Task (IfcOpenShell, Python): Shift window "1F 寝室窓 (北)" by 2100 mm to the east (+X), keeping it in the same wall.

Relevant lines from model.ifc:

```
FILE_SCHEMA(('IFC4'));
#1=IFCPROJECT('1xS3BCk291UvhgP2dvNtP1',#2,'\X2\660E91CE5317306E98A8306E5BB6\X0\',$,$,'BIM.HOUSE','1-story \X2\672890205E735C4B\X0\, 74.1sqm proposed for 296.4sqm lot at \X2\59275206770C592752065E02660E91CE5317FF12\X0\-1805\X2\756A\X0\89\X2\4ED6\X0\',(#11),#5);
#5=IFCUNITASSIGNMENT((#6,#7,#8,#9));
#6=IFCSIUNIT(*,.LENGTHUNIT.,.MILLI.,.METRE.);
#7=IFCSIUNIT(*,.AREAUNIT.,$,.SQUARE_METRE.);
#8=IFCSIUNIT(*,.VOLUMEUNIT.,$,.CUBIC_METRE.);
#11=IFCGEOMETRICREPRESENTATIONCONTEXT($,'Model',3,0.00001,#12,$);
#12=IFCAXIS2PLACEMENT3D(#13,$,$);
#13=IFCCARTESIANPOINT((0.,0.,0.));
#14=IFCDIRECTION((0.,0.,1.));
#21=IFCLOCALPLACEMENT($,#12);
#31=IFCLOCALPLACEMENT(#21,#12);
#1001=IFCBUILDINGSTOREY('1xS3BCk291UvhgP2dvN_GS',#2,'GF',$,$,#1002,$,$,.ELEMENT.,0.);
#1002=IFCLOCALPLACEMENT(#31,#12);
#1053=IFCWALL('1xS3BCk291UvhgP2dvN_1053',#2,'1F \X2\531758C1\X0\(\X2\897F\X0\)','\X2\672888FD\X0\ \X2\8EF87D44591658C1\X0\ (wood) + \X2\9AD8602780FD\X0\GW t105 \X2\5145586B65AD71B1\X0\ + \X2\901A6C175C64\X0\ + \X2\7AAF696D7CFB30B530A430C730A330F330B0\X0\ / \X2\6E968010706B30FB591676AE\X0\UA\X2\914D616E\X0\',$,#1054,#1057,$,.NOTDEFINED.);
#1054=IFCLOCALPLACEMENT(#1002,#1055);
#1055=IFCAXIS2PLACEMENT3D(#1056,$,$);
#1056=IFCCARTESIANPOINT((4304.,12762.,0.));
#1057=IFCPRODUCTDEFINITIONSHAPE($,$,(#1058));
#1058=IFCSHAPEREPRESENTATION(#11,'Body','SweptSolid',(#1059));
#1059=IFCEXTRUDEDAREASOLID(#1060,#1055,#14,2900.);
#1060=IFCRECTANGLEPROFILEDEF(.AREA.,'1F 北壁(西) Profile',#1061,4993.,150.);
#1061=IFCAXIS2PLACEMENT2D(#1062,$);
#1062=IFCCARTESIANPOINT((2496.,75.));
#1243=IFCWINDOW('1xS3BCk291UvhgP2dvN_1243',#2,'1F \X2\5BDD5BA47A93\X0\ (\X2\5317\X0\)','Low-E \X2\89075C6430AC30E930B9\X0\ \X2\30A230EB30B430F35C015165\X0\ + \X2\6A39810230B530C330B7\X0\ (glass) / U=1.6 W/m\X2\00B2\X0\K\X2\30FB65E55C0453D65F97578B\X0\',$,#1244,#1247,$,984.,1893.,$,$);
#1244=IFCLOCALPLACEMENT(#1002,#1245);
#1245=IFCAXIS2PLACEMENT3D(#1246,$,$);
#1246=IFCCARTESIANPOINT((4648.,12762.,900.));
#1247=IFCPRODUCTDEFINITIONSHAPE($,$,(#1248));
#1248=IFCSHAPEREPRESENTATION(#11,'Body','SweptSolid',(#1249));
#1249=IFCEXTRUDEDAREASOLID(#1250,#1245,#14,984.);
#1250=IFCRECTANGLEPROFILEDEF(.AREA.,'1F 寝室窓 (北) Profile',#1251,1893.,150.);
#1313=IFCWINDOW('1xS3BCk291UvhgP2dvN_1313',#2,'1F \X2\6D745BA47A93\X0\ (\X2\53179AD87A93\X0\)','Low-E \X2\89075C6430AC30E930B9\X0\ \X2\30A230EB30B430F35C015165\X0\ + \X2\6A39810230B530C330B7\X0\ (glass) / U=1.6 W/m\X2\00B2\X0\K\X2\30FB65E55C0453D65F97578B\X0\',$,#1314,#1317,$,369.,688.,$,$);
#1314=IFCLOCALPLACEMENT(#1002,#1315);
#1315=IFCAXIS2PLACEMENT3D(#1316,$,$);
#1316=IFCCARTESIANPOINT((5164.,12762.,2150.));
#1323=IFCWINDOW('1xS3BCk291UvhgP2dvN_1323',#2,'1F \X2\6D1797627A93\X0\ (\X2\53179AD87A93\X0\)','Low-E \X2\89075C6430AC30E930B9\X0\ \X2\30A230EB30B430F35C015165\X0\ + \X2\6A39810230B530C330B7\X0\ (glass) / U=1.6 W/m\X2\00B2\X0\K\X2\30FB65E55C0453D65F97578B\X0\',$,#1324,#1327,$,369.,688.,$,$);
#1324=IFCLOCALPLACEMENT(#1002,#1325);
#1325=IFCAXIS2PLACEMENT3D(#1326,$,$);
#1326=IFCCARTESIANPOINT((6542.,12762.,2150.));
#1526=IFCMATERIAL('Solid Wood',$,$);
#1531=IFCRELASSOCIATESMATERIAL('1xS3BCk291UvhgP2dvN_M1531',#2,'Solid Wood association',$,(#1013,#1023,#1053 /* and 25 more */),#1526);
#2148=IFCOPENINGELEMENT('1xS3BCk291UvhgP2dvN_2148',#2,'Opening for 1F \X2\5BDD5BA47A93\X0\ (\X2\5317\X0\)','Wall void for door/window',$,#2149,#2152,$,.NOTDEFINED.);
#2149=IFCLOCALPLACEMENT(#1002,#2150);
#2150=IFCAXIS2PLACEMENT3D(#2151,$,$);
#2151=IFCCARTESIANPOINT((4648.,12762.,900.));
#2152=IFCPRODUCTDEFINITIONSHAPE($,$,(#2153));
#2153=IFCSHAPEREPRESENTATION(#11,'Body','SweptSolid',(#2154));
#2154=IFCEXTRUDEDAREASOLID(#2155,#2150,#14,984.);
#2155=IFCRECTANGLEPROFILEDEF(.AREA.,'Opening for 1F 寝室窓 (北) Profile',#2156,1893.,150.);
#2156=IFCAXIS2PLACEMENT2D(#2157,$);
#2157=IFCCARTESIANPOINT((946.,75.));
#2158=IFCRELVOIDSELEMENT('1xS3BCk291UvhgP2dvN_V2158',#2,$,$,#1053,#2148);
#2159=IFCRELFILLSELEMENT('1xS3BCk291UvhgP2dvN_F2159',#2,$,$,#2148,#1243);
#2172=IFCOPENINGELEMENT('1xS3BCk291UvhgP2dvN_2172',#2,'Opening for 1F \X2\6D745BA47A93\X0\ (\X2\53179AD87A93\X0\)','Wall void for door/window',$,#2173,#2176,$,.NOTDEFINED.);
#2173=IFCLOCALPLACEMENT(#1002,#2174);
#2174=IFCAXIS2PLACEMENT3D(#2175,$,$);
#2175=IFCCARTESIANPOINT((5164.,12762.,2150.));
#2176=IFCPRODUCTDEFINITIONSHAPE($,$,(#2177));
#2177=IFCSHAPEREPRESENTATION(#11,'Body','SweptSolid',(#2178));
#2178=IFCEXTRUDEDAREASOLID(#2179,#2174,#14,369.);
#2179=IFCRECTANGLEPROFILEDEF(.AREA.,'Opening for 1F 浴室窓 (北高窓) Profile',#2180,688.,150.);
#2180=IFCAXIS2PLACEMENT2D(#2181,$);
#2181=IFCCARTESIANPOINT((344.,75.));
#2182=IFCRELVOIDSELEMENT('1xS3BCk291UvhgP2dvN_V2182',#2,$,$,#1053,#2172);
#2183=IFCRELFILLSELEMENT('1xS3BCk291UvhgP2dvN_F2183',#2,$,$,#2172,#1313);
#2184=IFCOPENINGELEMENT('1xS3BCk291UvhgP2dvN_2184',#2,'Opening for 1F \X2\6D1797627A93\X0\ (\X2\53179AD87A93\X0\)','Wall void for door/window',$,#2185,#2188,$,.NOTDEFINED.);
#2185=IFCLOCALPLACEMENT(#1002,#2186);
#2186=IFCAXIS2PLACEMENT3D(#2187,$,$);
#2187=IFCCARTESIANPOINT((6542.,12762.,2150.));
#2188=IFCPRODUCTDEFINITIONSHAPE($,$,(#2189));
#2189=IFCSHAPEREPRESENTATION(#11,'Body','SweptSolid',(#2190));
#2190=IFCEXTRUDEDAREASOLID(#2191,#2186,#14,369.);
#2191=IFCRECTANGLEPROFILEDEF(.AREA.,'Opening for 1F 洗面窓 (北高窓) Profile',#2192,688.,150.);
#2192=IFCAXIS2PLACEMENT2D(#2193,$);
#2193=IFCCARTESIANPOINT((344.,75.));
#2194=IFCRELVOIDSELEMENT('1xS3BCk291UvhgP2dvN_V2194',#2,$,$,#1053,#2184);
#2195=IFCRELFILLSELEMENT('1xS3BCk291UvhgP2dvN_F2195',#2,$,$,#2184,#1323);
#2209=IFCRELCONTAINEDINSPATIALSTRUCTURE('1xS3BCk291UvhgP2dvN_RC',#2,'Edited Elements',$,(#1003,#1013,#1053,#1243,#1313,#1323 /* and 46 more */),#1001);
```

```python
import ifcopenshell
import ifcopenshell.api.geometry
import ifcopenshell.util.placement
import ifcopenshell.util.unit

model = ifcopenshell.open("model.ifc")
unit_scale = ifcopenshell.util.unit.calculate_unit_scale(model)

window = model.by_id(1243)
opening = window.FillsVoids[0].RelatingOpeningElement
wall = opening.VoidsElements[0].RelatingBuildingElement

wall_matrix = ifcopenshell.util.placement.get_local_placement(wall.ObjectPlacement)
shift = wall_matrix[:3, 0] * 2.1 / unit_scale
before = ifcopenshell.util.placement.get_local_placement(window.ObjectPlacement)[:3, 3].copy()

# The window is not placed relative to its opening, so move both.
for product in (opening, window):
    matrix = ifcopenshell.util.placement.get_local_placement(product.ObjectPlacement)
    matrix[:3, 3] += shift
    ifcopenshell.api.geometry.edit_object_placement(model, product=product, matrix=matrix, is_si=False)

after = ifcopenshell.util.placement.get_local_placement(window.ObjectPlacement)[:3, 3]
print("window moved by", (after - before).round(3) + 0.0)

model.write("model-out.ifc")
```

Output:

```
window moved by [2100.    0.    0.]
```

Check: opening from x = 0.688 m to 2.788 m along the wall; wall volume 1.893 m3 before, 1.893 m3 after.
